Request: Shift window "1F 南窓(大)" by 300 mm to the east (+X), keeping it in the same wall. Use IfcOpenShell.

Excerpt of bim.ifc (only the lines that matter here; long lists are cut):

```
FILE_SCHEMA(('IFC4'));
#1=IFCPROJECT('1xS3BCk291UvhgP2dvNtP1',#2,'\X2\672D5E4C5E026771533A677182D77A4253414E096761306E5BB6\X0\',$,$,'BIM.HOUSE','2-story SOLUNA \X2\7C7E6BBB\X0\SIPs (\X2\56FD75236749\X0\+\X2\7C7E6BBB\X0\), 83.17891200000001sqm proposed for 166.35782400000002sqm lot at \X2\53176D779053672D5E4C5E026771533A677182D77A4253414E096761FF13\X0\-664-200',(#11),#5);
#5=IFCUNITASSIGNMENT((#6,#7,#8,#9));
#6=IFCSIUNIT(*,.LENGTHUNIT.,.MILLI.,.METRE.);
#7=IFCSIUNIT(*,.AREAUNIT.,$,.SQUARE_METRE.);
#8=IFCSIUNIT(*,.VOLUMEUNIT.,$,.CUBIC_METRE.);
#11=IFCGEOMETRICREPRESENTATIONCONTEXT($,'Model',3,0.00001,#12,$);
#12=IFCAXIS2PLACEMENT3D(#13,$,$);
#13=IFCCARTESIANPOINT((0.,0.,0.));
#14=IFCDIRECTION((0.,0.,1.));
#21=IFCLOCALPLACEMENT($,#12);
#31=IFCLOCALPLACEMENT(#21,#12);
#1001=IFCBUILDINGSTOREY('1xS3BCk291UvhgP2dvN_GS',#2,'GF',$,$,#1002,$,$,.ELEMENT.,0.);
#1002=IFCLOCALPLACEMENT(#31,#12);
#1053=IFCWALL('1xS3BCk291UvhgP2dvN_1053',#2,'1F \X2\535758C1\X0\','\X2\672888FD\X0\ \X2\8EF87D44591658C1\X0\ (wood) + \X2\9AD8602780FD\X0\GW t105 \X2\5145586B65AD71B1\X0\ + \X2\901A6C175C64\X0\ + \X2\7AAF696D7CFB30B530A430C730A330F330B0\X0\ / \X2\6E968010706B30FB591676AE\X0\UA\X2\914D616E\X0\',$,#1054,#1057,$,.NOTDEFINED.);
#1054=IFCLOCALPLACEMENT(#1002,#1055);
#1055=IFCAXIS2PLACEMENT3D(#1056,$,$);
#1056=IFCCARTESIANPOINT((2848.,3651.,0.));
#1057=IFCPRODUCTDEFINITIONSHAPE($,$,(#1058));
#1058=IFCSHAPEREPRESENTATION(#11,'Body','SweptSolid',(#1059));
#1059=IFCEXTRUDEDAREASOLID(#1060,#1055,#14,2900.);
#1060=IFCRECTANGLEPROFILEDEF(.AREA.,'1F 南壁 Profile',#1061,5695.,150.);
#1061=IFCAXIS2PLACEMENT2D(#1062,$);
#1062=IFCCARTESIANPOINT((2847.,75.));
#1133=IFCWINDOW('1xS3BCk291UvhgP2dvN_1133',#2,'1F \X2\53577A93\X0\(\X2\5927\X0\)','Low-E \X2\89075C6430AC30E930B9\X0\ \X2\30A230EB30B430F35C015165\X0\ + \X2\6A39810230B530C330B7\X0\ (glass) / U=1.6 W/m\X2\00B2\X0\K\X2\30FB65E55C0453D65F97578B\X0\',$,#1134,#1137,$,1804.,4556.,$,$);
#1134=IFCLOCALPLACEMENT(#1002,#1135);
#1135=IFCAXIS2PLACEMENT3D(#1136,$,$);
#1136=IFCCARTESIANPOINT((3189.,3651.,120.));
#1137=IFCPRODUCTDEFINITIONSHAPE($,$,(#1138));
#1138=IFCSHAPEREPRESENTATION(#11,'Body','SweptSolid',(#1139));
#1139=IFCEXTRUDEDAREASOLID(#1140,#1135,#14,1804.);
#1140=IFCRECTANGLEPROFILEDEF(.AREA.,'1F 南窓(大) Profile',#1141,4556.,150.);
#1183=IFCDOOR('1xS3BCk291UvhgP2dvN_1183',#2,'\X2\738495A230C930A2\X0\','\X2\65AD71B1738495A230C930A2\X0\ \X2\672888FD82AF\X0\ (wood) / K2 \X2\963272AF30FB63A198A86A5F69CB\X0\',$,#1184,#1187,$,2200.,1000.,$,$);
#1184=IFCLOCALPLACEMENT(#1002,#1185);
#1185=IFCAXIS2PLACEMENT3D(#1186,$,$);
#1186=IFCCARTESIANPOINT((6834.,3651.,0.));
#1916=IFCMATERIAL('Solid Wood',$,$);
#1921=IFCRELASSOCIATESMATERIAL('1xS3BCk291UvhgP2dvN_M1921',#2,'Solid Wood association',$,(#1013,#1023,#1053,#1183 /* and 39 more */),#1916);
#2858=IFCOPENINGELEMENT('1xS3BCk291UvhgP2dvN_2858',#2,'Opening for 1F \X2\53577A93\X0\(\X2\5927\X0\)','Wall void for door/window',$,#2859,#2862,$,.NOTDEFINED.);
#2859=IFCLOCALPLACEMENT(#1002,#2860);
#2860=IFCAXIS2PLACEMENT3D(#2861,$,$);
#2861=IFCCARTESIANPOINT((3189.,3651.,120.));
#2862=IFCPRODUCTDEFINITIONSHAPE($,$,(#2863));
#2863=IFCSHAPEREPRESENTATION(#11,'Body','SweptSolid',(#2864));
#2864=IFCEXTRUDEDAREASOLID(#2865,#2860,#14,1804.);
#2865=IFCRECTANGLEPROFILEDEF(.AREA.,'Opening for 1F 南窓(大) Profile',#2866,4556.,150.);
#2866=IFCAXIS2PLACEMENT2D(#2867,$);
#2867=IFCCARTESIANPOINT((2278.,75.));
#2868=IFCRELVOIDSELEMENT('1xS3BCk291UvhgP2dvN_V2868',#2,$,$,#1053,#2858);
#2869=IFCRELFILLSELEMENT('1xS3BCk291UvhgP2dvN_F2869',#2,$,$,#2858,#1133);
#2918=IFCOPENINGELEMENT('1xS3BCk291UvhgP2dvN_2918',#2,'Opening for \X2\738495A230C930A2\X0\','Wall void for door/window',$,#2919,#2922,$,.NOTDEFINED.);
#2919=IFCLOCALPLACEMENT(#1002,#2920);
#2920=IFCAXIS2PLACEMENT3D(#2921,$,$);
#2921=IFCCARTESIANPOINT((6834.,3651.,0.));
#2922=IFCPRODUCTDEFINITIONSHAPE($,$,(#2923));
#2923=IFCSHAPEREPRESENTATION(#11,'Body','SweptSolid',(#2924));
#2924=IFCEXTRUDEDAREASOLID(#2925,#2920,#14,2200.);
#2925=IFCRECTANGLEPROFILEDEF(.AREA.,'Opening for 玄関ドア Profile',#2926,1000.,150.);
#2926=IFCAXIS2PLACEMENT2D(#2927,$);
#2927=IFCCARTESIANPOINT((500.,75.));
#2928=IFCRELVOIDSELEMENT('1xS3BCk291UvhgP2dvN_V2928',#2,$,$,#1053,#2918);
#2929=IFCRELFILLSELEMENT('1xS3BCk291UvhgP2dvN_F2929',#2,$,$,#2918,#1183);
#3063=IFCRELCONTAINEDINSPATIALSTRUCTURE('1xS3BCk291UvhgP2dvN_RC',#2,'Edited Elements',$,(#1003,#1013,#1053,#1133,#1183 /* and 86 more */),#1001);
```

```python
import ifcopenshell
import ifcopenshell.api.geometry
import ifcopenshell.util.placement
import ifcopenshell.util.unit

model = ifcopenshell.open("bim.ifc")
unit_scale = ifcopenshell.util.unit.calculate_unit_scale(model)

window = model.by_guid("1xS3BCk291UvhgP2dvN_1133")
opening = window.FillsVoids[0].RelatingOpeningElement
wall = opening.VoidsElements[0].RelatingBuildingElement

wall_matrix = ifcopenshell.util.placement.get_local_placement(wall.ObjectPlacement)
shift = wall_matrix[:3, 0] * 0.3 / unit_scale
before = ifcopenshell.util.placement.get_local_placement(window.ObjectPlacement)[:3, 3].copy()

# The window is not placed relative to its opening, so move both.
for product in (opening, window):
    matrix = ifcopenshell.util.placement.get_local_placement(product.ObjectPlacement)
    matrix[:3, 3] += shift
    ifcopenshell.api.geometry.edit_object_placement(model, product=product, matrix=matrix, is_si=False)

after = ifcopenshell.util.placement.get_local_placement(window.ObjectPlacement)[:3, 3]
print("window moved by", (after - before).round(3) + 0.0)

model.write("bim_updated.ifc")
```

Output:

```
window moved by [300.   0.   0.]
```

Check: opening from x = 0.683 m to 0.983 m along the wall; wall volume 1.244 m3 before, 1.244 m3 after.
